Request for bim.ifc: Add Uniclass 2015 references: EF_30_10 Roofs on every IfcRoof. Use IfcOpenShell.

First a look at what the model holds.

```python
import ifcopenshell

model = ifcopenshell.open("bim.ifc")
print(model.schema)
print("classifications:", [c.Name for c in model.by_type("IfcClassification")])
for ifc_class in ("IfcDoor", "IfcRoof", "IfcStair", "IfcWall", "IfcWindow"):
    print(ifc_class, len(model.by_type(ifc_class)))
```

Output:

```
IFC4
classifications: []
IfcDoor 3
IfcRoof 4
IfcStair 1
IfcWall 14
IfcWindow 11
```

```python
import ifcopenshell
import ifcopenshell.api.classification

model = ifcopenshell.open("bim.ifc")

system = ifcopenshell.api.classification.add_classification(model, classification="Uniclass 2015")

codes = {
    "IfcRoof": ("EF_30_10", "Roofs"),
}
for ifc_class, (code, name) in codes.items():
    products = model.by_type(ifc_class)
    ifcopenshell.api.classification.add_reference(
        model, products=products, classification=system, identification=code, name=name
    )
    print(code, len(products))

model.write("bim_rev.ifc")
```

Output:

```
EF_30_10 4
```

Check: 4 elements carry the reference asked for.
